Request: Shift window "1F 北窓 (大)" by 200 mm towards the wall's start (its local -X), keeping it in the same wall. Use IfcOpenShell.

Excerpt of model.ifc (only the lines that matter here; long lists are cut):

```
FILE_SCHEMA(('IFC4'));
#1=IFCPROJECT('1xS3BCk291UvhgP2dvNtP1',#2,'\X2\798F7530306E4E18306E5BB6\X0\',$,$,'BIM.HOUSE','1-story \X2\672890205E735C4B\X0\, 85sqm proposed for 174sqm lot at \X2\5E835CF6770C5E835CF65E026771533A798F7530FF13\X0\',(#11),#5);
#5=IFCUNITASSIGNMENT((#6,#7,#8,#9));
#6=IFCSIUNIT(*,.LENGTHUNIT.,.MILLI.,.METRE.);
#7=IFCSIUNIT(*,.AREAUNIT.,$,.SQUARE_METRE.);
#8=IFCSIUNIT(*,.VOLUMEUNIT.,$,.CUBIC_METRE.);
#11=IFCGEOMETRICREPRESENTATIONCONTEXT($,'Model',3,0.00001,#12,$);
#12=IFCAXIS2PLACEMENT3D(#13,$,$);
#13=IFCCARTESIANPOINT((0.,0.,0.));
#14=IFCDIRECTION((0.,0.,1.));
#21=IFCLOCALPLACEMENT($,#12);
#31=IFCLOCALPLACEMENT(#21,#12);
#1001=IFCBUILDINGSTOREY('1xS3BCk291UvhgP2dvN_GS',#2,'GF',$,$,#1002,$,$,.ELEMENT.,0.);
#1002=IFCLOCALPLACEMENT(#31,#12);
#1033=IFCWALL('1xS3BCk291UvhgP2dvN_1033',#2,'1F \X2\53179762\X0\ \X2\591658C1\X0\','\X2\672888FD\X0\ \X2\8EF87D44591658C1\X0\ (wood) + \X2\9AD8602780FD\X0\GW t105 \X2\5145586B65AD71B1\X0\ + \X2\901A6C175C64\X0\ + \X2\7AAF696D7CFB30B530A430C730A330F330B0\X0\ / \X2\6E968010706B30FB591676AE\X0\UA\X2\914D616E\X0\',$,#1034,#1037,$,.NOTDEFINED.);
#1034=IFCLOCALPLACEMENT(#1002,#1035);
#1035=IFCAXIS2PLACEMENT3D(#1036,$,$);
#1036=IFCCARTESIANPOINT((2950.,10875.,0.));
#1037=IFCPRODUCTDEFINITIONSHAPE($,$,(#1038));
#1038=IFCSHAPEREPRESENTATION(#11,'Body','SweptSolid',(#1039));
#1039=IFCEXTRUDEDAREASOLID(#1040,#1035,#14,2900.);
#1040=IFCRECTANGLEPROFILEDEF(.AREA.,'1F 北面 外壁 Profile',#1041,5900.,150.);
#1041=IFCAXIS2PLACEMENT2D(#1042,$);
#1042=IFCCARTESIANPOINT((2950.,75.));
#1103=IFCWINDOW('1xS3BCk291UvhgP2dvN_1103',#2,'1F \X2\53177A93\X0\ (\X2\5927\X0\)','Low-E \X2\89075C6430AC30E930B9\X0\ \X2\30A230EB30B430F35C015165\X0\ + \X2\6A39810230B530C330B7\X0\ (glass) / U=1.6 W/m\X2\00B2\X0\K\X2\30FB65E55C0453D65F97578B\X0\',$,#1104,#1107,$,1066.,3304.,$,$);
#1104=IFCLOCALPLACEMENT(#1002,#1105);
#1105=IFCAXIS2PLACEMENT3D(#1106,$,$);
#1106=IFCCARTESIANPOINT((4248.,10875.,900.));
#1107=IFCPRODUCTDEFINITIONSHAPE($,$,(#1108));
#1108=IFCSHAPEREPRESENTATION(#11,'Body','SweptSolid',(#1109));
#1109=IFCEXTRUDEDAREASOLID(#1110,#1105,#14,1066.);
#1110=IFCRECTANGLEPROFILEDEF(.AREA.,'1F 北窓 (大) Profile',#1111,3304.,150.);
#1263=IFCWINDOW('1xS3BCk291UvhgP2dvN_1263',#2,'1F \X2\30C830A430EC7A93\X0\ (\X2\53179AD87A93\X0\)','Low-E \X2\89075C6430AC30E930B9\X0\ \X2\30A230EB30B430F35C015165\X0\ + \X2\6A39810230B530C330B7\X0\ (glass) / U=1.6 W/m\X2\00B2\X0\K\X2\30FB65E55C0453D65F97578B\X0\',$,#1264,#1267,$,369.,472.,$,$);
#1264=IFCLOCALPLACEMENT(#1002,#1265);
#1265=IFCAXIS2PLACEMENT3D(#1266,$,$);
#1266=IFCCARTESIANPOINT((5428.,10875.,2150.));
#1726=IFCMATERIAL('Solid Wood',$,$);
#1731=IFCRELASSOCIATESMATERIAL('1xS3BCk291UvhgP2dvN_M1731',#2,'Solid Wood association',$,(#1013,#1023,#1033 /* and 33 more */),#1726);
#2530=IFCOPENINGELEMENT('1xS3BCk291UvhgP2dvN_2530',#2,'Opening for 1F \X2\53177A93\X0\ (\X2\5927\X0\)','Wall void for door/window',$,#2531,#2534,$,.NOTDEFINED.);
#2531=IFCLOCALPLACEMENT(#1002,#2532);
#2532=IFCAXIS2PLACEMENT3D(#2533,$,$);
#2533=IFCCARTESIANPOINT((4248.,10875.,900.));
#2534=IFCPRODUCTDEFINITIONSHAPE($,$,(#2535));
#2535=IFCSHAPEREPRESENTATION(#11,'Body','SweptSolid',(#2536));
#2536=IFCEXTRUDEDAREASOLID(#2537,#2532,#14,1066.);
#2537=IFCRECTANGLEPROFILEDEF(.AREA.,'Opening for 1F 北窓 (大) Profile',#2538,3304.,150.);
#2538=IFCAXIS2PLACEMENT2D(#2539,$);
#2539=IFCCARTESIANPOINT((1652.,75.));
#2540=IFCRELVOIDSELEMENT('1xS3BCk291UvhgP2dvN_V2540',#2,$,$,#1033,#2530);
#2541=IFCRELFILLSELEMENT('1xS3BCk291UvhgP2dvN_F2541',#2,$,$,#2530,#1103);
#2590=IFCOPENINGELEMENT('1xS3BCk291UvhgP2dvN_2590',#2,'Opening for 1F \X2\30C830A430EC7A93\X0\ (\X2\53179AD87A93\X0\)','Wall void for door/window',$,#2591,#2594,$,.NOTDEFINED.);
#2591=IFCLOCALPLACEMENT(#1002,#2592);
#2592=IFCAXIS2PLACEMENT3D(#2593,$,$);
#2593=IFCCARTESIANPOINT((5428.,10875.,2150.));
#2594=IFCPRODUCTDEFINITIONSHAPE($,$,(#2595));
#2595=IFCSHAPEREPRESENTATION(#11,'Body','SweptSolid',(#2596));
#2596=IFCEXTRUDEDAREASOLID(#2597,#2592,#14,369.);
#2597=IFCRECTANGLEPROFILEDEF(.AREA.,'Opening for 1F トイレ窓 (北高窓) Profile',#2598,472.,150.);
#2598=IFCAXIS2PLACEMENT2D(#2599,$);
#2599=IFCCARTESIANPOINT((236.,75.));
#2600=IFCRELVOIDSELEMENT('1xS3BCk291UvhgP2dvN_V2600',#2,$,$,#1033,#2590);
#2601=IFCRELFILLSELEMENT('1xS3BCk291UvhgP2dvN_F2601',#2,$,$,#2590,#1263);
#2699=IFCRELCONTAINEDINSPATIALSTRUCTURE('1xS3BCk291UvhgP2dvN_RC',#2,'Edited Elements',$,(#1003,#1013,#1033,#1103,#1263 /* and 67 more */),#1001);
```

```python
import ifcopenshell
import ifcopenshell.api.geometry
import ifcopenshell.util.placement

model = ifcopenshell.open("model.ifc")

window = model.by_guid("1xS3BCk291UvhgP2dvN_1103")
opening = window.FillsVoids[0].RelatingOpeningElement
wall = opening.VoidsElements[0].RelatingBuildingElement

wall_matrix = ifcopenshell.util.placement.get_local_placement(wall.ObjectPlacement)
shift = wall_matrix[:3, 0] * -200.0
before = ifcopenshell.util.placement.get_local_placement(window.ObjectPlacement)[:3, 3].copy()

# The window is not placed relative to its opening, so move both.
for product in (opening, window):
    matrix = ifcopenshell.util.placement.get_local_placement(product.ObjectPlacement)
    matrix[:3, 3] += shift
    ifcopenshell.api.geometry.edit_object_placement(model, product=product, matrix=matrix, is_si=False)

after = ifcopenshell.util.placement.get_local_placement(window.ObjectPlacement)[:3, 3]
print("window moved by", (after - before).round(3) + 0.0)

model.write("model_v2.ifc")
```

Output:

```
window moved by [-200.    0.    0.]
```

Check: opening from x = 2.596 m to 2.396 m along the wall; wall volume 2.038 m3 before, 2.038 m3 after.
